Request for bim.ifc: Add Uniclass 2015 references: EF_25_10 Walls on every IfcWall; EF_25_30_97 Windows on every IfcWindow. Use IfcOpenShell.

First a look at what the model holds.

```python
import ifcopenshell

model = ifcopenshell.open("bim.ifc")
print(model.schema)
print("classifications:", [c.Name for c in model.by_type("IfcClassification")])
for ifc_class in ("IfcDoor", "IfcRoof", "IfcStair", "IfcWall", "IfcWindow"):
    print(ifc_class, len(model.by_type(ifc_class)))
```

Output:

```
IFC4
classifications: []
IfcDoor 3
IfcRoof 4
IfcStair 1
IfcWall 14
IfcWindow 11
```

```python
import ifcopenshell
import ifcopenshell.api.classification

model = ifcopenshell.open("bim.ifc")

system = ifcopenshell.api.classification.add_classification(model, classification="Uniclass 2015")

codes = {
    "IfcWall": ("EF_25_10", "Walls"),
    "IfcWindow": ("EF_25_30_97", "Windows"),
}
for ifc_class, (code, name) in codes.items():
    products = model.by_type(ifc_class)
    ifcopenshell.api.classification.add_reference(
        model, products=products, classification=system, identification=code, name=name
    )
    print(code, len(products))

model.write("bim-out.ifc")
```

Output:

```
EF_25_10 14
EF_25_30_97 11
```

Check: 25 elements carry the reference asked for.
